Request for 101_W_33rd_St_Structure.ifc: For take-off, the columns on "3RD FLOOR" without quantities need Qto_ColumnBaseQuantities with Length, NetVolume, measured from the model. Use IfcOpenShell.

First a look at what the model holds.

```python
import ifcopenshell
import ifcopenshell.util.element
import ifcopenshell.util.unit

model = ifcopenshell.open("101_W_33rd_St_Structure.ifc")
print(model.schema)
for unit_type in ("LENGTHUNIT", "AREAUNIT", "VOLUMEUNIT"):
    print(unit_type, ifcopenshell.util.unit.calculate_unit_scale(model, unit_type))
storey = next(s for s in model.by_type("IfcBuildingStorey") if s.Name == "3RD FLOOR")
columns = [e for e in ifcopenshell.util.element.get_decomposition(storey) if e.is_a("IfcColumn")]
for e in sorted(columns, key=lambda e: e.id()):
    print(e.id(), e.is_a(), e.Name, list(ifcopenshell.util.element.get_psets(e, qtos_only=True)), sep=" | ")
```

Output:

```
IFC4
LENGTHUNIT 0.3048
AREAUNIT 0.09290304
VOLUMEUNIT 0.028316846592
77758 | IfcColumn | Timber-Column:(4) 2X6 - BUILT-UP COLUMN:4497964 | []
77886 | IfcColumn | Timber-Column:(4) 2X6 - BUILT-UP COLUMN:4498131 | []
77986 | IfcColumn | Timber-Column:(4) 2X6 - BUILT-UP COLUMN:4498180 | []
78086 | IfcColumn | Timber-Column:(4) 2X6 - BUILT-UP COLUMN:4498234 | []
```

```python
import ifcopenshell
import ifcopenshell.api.pset
import ifcopenshell.geom
import ifcopenshell.util.element
import ifcopenshell.util.shape
import ifcopenshell.util.unit

model = ifcopenshell.open("101_W_33rd_St_Structure.ifc")
unit_scale = ifcopenshell.util.unit.calculate_unit_scale(model)
volume_scale = ifcopenshell.util.unit.calculate_unit_scale(model, "VOLUMEUNIT")
settings = ifcopenshell.geom.settings()

storey = next(s for s in model.by_type("IfcBuildingStorey") if s.Name == "3RD FLOOR")
columns = [e for e in ifcopenshell.util.element.get_decomposition(storey) if e.is_a("IfcColumn")]

for e in sorted(columns, key=lambda e: e.id()):
    if ifcopenshell.util.element.get_psets(e, qtos_only=True, should_inherit=False):
        continue
    # Geometry comes back in metres, in the element's own axes.
    shape = ifcopenshell.geom.create_shape(settings, e)
    values = {
        "Length": ifcopenshell.util.shape.get_z(shape.geometry) / unit_scale,
        "NetVolume": ifcopenshell.util.shape.get_volume(shape.geometry) / volume_scale,
    }
    qto = ifcopenshell.api.pset.add_qto(model, product=e, name="Qto_ColumnBaseQuantities")
    ifcopenshell.api.pset.edit_qto(model, qto=qto, properties=values)
    print(e.id(), {k: round(v, 3) for k, v in values.items()})

model.write("101_W_33rd_St_Structure_rev.ifc")
```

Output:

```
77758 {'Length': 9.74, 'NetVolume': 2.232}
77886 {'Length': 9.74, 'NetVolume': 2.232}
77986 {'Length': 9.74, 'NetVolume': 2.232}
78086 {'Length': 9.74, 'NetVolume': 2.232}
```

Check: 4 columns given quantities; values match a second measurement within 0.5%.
